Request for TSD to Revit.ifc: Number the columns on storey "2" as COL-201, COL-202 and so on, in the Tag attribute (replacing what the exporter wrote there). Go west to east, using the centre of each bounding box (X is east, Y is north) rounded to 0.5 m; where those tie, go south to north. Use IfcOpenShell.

First a look at what the model holds.

```python
import ifcopenshell
import ifcopenshell.util.element
import ifcopenshell.util.placement

model = ifcopenshell.open("TSD to Revit.ifc")
print(model.schema)
storey = next(s for s in model.by_type("IfcBuildingStorey") if s.Name == "2")
columns = [e for e in ifcopenshell.util.element.get_decomposition(storey) if e.is_a("IfcColumn")]
for e in sorted(columns, key=lambda e: e.id()):
    origin = ifcopenshell.util.placement.get_local_placement(e.ObjectPlacement)[:3, 3]
    print(e.id(), e.Tag, e.Name, origin.round(2) + 0.0, sep=" | ")
```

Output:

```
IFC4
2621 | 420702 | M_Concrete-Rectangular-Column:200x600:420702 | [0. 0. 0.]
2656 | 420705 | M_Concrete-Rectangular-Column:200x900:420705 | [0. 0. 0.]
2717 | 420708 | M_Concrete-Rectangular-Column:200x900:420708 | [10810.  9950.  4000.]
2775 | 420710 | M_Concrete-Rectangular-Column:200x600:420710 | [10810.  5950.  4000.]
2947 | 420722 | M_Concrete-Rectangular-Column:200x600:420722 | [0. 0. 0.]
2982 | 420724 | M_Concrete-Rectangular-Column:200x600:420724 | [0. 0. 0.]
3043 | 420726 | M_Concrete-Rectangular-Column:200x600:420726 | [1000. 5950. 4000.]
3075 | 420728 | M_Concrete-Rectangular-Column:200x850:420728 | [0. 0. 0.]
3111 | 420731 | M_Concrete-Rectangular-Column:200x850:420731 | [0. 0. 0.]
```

```python
import ifcopenshell
import ifcopenshell.geom
import ifcopenshell.util.element
import ifcopenshell.util.shape

model = ifcopenshell.open("TSD to Revit.ifc")
settings = ifcopenshell.geom.settings()
settings.set("use-world-coords", True)


def centre(element):
    shape = ifcopenshell.geom.create_shape(settings, element)
    return ifcopenshell.util.shape.get_bbox_centroid(shape.geometry)


storey = next(s for s in model.by_type("IfcBuildingStorey") if s.Name == "2")
columns = [e for e in ifcopenshell.util.element.get_decomposition(storey) if e.is_a("IfcColumn")]

# Insertion points can sit at a corner or the storey origin, so sort by the geometry (in metres).
centres = {e: centre(e) for e in columns}
columns.sort(key=lambda e: (round(centres[e][0] / 0.5), centres[e][1]))

for i, e in enumerate(columns, start=1):
    number = f"COL-2{i:02d}"
    e.Tag = number
    print(e.id(), number)

model.write("TSD to Revit-out.ifc")
```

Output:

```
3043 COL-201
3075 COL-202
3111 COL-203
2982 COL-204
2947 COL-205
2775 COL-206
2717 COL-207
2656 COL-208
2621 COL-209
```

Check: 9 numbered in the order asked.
